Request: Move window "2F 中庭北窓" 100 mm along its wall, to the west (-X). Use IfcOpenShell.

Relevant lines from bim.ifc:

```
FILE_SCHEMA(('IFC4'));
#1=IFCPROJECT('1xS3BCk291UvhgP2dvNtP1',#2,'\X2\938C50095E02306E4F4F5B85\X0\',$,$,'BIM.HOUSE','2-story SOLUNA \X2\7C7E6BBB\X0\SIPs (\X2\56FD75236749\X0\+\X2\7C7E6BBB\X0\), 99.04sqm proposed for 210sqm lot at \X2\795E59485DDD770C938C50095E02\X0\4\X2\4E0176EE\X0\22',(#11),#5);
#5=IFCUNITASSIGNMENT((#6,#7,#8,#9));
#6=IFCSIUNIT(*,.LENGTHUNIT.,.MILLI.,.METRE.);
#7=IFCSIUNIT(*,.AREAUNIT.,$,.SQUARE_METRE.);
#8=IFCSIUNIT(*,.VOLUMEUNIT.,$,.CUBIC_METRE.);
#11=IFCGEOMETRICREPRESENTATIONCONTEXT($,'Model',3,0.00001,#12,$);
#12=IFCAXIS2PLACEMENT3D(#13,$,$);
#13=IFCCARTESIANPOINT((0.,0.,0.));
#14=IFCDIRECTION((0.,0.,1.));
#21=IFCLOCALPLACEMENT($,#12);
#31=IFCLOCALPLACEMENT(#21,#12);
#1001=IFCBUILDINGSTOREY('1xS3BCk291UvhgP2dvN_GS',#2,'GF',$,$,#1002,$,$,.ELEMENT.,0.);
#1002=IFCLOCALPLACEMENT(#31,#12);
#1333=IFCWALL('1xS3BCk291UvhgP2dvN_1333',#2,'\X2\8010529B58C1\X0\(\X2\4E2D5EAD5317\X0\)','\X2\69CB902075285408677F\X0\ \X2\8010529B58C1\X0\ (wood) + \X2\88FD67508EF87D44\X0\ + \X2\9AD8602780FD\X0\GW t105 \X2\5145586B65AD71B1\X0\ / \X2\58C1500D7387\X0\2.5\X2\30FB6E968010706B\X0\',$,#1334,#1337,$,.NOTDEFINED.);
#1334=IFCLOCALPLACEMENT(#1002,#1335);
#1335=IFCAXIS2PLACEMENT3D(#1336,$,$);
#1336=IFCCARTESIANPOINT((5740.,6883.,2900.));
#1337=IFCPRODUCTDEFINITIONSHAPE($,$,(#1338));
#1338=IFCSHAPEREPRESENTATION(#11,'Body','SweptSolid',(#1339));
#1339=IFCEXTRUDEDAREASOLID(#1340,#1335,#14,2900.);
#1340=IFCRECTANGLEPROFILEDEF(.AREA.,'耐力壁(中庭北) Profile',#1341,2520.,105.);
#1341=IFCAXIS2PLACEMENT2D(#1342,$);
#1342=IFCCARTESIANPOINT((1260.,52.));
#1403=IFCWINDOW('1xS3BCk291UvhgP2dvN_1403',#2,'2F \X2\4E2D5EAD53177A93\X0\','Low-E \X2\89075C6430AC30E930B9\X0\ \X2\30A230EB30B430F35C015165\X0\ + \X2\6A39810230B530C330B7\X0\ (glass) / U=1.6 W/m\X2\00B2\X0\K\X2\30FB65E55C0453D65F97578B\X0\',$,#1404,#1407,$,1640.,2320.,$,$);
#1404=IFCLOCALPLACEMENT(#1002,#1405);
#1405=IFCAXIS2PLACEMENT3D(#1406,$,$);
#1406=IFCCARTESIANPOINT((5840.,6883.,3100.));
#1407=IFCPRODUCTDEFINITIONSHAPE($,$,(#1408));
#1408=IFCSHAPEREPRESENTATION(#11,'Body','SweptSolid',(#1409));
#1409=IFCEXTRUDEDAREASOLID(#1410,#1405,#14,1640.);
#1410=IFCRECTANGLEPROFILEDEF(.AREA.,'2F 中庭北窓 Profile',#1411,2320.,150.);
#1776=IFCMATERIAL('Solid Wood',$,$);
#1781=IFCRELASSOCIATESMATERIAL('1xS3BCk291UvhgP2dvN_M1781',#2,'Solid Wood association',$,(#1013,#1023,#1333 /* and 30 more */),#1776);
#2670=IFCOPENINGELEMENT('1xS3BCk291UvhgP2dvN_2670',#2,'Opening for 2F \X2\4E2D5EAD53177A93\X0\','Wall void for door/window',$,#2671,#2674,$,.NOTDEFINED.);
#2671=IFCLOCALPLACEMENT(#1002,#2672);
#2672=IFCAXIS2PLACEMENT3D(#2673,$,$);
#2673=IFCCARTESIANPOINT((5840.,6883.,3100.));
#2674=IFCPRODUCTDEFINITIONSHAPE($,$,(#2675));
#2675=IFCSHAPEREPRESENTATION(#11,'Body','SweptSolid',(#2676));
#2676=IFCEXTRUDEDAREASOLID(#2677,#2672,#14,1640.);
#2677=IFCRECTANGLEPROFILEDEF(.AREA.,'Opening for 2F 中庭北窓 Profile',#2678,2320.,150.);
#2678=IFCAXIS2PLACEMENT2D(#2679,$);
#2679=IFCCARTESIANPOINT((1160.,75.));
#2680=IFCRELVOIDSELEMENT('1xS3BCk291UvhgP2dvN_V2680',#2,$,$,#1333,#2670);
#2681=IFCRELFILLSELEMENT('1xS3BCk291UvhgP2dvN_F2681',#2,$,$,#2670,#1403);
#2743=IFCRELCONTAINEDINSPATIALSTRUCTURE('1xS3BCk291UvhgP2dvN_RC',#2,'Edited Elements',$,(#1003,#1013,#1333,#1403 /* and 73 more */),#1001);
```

```python
import ifcopenshell
import ifcopenshell.api.geometry
import ifcopenshell.util.placement

model = ifcopenshell.open("bim.ifc")

window = model.by_guid("1xS3BCk291UvhgP2dvN_1403")
opening = window.FillsVoids[0].RelatingOpeningElement
wall = opening.VoidsElements[0].RelatingBuildingElement

wall_matrix = ifcopenshell.util.placement.get_local_placement(wall.ObjectPlacement)
shift = wall_matrix[:3, 0] * -100.0
before = ifcopenshell.util.placement.get_local_placement(window.ObjectPlacement)[:3, 3].copy()

# The window is not placed relative to its opening, so move both.
for product in (opening, window):
    matrix = ifcopenshell.util.placement.get_local_placement(product.ObjectPlacement)
    matrix[:3, 3] += shift
    ifcopenshell.api.geometry.edit_object_placement(model, product=product, matrix=matrix, is_si=False)

after = ifcopenshell.util.placement.get_local_placement(window.ObjectPlacement)[:3, 3]
print("window moved by", (after - before).round(3) + 0.0)

model.write("bim_v2.ifc")
```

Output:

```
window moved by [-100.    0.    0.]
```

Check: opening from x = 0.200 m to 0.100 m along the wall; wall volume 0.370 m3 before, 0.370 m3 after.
